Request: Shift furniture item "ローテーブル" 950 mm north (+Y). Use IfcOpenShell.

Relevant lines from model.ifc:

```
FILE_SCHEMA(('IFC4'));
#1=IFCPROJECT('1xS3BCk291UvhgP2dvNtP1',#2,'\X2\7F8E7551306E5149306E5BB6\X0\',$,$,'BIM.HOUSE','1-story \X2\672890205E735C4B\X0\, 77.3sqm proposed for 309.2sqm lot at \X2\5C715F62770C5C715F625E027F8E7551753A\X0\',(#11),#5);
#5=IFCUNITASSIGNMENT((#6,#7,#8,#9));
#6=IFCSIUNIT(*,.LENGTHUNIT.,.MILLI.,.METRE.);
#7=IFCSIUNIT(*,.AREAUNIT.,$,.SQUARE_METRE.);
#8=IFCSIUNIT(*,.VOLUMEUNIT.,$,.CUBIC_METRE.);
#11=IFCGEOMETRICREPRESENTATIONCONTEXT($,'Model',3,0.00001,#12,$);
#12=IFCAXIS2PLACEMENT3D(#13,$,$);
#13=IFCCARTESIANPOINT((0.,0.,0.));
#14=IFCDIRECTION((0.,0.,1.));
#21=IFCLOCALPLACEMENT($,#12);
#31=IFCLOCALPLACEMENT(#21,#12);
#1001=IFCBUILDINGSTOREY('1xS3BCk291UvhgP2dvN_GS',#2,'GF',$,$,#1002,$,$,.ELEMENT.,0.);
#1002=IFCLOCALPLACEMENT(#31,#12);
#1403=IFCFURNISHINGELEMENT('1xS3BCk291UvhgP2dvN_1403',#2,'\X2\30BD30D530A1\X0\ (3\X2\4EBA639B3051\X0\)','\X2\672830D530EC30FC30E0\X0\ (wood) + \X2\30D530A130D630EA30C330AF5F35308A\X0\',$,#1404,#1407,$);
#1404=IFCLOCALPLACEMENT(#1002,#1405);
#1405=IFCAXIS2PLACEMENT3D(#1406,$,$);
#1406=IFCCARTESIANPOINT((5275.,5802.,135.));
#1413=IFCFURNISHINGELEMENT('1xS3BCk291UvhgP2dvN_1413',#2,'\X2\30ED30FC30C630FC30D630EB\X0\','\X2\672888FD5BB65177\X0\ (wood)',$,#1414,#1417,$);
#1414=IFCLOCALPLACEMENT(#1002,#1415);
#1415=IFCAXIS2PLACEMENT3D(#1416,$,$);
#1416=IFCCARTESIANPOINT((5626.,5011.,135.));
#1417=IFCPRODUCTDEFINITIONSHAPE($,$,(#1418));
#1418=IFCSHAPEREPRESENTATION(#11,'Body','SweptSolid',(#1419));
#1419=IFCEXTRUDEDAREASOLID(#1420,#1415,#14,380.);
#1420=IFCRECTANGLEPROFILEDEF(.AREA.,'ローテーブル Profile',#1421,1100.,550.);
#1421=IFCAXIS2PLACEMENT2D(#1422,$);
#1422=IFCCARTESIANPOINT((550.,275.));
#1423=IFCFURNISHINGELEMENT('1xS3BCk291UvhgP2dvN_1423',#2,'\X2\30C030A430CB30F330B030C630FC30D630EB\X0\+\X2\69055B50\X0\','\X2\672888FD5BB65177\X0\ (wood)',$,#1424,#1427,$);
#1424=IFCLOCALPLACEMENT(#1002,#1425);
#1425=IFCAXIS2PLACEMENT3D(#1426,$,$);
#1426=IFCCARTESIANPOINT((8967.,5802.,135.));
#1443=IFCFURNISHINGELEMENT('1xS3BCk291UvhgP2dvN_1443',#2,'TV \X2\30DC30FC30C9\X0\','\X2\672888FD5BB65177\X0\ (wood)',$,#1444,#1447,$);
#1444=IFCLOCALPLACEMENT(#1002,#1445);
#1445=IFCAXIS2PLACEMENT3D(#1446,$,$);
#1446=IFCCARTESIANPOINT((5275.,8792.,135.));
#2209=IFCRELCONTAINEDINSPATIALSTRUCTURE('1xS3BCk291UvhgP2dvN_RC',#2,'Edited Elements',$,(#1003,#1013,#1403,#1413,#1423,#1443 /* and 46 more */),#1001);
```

```python
import ifcopenshell
import ifcopenshell.api.geometry
import ifcopenshell.util.placement
import ifcopenshell.util.unit

model = ifcopenshell.open("model.ifc")
unit_scale = ifcopenshell.util.unit.calculate_unit_scale(model)

item = model.by_guid("1xS3BCk291UvhgP2dvN_1413")
matrix = ifcopenshell.util.placement.get_local_placement(item.ObjectPlacement)
matrix[1, 3] += 0.95 / unit_scale
ifcopenshell.api.geometry.edit_object_placement(model, product=item, matrix=matrix, is_si=False)

print(ifcopenshell.util.placement.get_local_placement(item.ObjectPlacement).round(3) + 0.0)

model.write("model_rev.ifc")
```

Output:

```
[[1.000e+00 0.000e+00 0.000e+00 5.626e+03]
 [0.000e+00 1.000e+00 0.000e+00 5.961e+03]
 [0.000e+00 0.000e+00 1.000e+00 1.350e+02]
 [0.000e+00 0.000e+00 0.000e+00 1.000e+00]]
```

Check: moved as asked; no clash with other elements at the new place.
